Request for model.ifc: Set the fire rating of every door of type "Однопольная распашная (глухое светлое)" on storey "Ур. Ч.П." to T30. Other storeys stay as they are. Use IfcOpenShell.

First a look at what the model holds.

```python
import ifcopenshell
import ifcopenshell.util.element

model = ifcopenshell.open("model.ifc")
print(model.schema)
storey = next(s for s in model.by_type("IfcBuildingStorey") if s.Name == "Ур. Ч.П.")
doors = [e for e in ifcopenshell.util.element.get_decomposition(storey) if e.is_a("IfcDoor")]
seen = {}
for e in doors:
    element_type = ifcopenshell.util.element.get_type(e)
    key = (element_type.Name if element_type != e and element_type else None, ifcopenshell.util.element.get_pset(e, "Pset_DoorCommon", "FireRating"))
    seen[key] = seen.get(key, 0) + 1
for (name, value), count in sorted(seen.items(), key=str):
    print(count, "x", name, "|", value)
```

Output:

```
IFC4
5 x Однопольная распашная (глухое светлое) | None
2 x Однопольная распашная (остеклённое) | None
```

```python
import ifcopenshell
import ifcopenshell.api.pset
import ifcopenshell.util.element

model = ifcopenshell.open("model.ifc")

storey = next(s for s in model.by_type("IfcBuildingStorey") if s.Name == "Ур. Ч.П.")
doors = [e for e in ifcopenshell.util.element.get_decomposition(storey) if e.is_a("IfcDoor")]

count = 0
for e in doors:
    element_type = ifcopenshell.util.element.get_type(e)
    if element_type in (None, e) or element_type.Name != "Однопольная распашная (глухое светлое)":
        continue
    # add_pset returns the element's existing set when there is one.
    pset = ifcopenshell.api.pset.add_pset(model, product=e, name="Pset_DoorCommon")
    ifcopenshell.api.pset.edit_pset(model, pset=pset, properties={"FireRating": "T30"})
    count += 1

print(count, "doors updated")

model.write("model_edited.ifc")
```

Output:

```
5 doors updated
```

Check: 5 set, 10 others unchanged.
